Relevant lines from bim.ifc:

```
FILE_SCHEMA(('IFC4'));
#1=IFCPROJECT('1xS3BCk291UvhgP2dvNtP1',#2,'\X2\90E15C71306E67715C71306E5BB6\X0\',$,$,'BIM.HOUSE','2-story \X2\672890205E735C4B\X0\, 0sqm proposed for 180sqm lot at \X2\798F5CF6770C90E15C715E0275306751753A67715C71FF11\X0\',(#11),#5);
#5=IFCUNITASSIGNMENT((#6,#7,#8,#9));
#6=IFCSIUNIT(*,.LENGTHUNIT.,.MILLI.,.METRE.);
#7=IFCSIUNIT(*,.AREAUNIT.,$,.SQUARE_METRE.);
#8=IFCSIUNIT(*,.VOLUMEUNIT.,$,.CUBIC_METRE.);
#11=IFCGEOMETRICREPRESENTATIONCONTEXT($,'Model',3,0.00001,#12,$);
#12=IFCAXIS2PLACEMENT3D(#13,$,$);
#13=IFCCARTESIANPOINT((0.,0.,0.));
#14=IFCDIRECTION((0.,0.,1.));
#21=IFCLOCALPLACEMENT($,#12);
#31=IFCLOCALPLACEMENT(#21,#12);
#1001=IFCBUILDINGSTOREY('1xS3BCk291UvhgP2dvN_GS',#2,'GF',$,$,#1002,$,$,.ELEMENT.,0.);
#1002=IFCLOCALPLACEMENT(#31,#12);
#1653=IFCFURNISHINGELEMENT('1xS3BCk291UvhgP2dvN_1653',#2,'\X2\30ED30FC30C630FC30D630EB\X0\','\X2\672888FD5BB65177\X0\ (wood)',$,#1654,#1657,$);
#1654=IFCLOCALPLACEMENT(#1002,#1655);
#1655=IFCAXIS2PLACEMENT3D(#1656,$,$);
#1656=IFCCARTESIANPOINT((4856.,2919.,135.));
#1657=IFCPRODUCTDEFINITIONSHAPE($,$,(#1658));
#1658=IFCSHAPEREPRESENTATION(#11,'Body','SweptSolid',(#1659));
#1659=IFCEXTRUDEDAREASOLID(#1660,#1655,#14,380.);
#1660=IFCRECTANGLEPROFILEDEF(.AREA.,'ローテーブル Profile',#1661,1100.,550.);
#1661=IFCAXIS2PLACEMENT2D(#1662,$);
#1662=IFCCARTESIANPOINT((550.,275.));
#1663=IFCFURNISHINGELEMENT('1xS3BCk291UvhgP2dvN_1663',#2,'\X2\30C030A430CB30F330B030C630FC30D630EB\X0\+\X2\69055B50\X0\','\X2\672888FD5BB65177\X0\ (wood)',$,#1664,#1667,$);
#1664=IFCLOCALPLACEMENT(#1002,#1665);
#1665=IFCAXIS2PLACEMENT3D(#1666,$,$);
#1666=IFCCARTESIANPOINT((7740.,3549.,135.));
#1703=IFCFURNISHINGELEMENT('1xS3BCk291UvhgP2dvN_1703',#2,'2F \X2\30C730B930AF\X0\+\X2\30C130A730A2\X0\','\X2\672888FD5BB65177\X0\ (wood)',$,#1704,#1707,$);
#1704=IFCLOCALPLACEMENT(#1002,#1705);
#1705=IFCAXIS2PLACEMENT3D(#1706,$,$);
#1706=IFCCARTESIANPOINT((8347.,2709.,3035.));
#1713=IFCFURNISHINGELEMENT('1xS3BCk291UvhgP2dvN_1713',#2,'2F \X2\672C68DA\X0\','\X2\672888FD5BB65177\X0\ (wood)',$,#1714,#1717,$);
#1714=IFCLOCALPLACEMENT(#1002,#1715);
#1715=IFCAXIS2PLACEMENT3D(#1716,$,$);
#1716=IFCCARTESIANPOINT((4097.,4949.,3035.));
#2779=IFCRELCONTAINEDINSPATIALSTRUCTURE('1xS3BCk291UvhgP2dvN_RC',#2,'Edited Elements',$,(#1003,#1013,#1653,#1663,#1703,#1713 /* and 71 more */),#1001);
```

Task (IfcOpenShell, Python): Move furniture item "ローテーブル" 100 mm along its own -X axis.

```python
import ifcopenshell
import ifcopenshell.api.geometry
import ifcopenshell.util.placement
import ifcopenshell.util.unit

model = ifcopenshell.open("bim.ifc")
unit_scale = ifcopenshell.util.unit.calculate_unit_scale(model)

item = model.by_guid("1xS3BCk291UvhgP2dvN_1653")
matrix = ifcopenshell.util.placement.get_local_placement(item.ObjectPlacement)
matrix[:3, 3] -= matrix[:3, 0] * 0.1 / unit_scale
ifcopenshell.api.geometry.edit_object_placement(model, product=item, matrix=matrix, is_si=False)

print(ifcopenshell.util.placement.get_local_placement(item.ObjectPlacement).round(3) + 0.0)

model.write("bim_edited.ifc")
```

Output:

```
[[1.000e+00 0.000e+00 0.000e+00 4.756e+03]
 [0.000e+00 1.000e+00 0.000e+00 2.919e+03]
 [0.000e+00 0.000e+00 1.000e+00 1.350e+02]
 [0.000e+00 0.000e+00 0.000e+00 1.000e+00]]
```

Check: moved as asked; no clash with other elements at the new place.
